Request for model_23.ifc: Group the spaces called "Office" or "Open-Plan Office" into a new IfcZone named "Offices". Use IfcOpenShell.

First a look at what the model holds.

```python
import ifcopenshell

model = ifcopenshell.open("model_23.ifc")
print(model.schema)
seen = {}
for space in model.by_type("IfcSpace"):
    seen[space.LongName] = seen.get(space.LongName, 0) + 1
for name, count in sorted(seen.items(), key=str):
    print(count, "x", name)
print("zones:", [z.Name for z in model.by_type("IfcZone")][:20])
```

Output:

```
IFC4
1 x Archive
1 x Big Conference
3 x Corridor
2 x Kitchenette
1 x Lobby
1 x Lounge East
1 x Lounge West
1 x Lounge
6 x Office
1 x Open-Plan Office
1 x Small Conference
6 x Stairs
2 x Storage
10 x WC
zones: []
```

```python
import ifcopenshell
import ifcopenshell.api.group
import ifcopenshell.api.root

model = ifcopenshell.open("model_23.ifc")

names = {"Office", "Open-Plan Office"}
spaces = [s for s in model.by_type("IfcSpace") if s.LongName in names]

zone = ifcopenshell.api.root.create_entity(model, ifc_class="IfcZone", name="Offices")
ifcopenshell.api.group.assign_group(model, products=spaces, group=zone)
print(len(spaces), "spaces in", zone.Name)

model.write("model_23_v2.ifc")
```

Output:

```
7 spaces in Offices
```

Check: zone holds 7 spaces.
